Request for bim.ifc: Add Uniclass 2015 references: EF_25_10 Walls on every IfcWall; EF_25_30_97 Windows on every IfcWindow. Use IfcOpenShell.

First a look at what the model holds.

```python
import ifcopenshell

model = ifcopenshell.open("bim.ifc")
print(model.schema)
print("classifications:", [c.Name for c in model.by_type("IfcClassification")])
for ifc_class in ("IfcDoor", "IfcRoof", "IfcStair", "IfcWall", "IfcWindow"):
    print(ifc_class, len(model.by_type(ifc_class)))
```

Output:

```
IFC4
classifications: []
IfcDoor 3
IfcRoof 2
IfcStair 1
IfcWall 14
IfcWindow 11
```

```python
import ifcopenshell
import ifcopenshell.api.classification

model = ifcopenshell.open("bim.ifc")

system = ifcopenshell.api.classification.add_classification(model, classification="Uniclass 2015")

codes = {
    "IfcWall": ("EF_25_10", "Walls"),
    "IfcWindow": ("EF_25_30_97", "Windows"),
}
for ifc_class, (code, name) in codes.items():
    products = model.by_type(ifc_class)
    ifcopenshell.api.classification.add_reference(
        model, products=products, classification=system, identification=code, name=name
    )
    print(code, len(products))

model.write("bim-out.ifc")
```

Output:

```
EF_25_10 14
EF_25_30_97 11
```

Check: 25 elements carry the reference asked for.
